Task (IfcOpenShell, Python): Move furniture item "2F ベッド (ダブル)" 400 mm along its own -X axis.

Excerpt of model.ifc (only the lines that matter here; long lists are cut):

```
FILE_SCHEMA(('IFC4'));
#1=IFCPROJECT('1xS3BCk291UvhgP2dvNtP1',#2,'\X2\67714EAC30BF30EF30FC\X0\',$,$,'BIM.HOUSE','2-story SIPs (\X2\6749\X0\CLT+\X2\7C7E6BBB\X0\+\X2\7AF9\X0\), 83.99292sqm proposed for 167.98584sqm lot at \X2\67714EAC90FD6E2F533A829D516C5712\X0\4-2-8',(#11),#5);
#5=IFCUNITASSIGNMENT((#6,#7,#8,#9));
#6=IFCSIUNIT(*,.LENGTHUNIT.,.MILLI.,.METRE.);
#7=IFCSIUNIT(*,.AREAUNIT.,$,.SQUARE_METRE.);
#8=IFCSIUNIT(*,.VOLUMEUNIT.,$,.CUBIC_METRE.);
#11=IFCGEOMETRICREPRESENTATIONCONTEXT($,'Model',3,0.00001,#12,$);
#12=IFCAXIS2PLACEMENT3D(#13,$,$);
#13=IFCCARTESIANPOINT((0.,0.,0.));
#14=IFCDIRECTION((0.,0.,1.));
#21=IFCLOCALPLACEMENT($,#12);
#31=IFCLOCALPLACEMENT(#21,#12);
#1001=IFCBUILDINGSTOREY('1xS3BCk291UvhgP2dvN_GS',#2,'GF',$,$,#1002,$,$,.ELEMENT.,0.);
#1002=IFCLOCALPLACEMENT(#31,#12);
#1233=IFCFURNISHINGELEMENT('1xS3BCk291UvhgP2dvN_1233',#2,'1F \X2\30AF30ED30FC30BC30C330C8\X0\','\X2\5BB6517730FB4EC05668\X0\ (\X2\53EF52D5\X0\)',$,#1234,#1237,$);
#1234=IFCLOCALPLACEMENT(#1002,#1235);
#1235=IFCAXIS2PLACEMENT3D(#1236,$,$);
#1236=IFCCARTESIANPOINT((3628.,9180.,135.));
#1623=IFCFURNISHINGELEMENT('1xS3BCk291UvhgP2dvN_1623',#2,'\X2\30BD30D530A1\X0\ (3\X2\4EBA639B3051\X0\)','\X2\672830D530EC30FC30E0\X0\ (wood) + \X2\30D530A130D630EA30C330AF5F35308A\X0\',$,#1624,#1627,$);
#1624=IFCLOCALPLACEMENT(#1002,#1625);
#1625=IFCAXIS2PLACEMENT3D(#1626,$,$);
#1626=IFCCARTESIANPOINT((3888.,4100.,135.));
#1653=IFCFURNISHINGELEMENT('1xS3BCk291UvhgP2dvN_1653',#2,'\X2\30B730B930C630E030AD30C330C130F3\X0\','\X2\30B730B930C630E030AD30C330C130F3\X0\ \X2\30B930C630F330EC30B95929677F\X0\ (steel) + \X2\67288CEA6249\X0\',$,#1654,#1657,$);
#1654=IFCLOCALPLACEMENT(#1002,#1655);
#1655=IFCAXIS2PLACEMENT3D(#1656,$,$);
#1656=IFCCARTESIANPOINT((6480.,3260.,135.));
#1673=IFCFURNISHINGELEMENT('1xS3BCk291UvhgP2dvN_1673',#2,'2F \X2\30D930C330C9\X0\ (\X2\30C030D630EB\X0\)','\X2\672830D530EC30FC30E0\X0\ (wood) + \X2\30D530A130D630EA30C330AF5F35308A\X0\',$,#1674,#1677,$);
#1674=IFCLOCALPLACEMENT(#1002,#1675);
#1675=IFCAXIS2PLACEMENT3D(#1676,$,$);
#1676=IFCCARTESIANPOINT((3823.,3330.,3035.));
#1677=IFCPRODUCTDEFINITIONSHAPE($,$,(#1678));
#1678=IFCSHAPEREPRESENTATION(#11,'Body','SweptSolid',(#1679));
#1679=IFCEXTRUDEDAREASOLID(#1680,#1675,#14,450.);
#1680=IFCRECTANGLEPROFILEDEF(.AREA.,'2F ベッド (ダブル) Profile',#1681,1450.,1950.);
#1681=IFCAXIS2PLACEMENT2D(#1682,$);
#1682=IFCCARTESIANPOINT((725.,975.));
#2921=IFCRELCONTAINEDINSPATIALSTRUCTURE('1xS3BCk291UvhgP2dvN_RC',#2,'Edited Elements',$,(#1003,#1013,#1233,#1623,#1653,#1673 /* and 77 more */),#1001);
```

```python
import ifcopenshell
import ifcopenshell.api.geometry
import ifcopenshell.util.placement
import ifcopenshell.util.unit

model = ifcopenshell.open("model.ifc")
unit_scale = ifcopenshell.util.unit.calculate_unit_scale(model)

item = model.by_guid("1xS3BCk291UvhgP2dvN_1673")
matrix = ifcopenshell.util.placement.get_local_placement(item.ObjectPlacement)
matrix[:3, 3] -= matrix[:3, 0] * 0.4 / unit_scale
ifcopenshell.api.geometry.edit_object_placement(model, product=item, matrix=matrix, is_si=False)

print(ifcopenshell.util.placement.get_local_placement(item.ObjectPlacement).round(3) + 0.0)

model.write("model_edited.ifc")
```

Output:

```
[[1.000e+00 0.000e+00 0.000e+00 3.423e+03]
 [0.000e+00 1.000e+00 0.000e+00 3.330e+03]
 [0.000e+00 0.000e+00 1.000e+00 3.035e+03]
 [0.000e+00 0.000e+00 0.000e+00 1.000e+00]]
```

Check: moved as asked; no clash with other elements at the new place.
